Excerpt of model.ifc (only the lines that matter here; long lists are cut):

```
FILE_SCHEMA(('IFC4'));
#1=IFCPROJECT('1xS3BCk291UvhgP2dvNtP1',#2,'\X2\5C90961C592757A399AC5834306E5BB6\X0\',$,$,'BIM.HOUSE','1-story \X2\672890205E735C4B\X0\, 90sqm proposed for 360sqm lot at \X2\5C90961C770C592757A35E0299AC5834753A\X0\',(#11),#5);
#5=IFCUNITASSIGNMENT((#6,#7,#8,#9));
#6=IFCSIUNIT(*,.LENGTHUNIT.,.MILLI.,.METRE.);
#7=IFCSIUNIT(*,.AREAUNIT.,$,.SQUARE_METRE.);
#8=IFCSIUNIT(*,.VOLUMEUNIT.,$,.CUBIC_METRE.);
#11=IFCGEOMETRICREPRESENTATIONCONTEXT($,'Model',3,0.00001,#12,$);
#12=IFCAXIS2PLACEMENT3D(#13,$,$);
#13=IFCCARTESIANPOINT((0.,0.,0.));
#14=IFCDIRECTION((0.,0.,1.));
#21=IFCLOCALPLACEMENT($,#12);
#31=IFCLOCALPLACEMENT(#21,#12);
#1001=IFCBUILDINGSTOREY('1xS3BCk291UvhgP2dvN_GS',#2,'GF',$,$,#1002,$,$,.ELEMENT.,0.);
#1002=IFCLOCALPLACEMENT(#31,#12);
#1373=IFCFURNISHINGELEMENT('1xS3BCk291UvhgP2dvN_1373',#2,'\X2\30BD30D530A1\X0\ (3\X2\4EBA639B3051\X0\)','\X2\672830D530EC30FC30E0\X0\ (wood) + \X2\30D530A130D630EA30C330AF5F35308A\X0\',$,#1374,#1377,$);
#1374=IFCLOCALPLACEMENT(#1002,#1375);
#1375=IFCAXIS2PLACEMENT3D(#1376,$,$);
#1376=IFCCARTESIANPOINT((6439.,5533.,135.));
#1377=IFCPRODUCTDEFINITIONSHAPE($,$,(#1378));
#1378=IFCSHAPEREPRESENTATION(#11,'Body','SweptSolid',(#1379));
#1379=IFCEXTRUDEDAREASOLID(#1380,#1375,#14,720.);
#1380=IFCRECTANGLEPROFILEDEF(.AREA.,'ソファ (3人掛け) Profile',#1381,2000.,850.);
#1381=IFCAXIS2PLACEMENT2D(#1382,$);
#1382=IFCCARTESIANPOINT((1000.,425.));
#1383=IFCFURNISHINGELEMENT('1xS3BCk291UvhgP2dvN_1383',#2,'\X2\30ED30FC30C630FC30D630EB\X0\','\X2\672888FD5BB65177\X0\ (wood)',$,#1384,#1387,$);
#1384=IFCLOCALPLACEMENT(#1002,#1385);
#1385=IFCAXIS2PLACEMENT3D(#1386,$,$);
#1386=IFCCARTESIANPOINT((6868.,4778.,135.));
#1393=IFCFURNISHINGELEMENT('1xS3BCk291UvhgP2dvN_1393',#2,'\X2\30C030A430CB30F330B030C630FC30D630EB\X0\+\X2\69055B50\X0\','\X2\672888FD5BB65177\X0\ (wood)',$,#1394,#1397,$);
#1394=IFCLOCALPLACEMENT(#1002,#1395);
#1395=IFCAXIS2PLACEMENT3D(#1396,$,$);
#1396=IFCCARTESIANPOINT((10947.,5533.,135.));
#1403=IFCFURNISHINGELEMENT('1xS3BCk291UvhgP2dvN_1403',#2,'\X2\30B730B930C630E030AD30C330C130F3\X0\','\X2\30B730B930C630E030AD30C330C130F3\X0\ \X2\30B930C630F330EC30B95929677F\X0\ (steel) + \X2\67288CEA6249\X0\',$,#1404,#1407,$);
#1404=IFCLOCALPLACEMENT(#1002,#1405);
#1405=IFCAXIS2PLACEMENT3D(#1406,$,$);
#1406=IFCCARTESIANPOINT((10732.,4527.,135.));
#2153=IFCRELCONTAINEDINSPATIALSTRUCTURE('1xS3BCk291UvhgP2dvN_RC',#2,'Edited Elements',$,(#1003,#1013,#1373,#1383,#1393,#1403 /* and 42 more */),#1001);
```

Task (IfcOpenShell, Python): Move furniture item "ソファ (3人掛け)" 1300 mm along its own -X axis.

```python
import ifcopenshell
import ifcopenshell.api.geometry
import ifcopenshell.util.placement

model = ifcopenshell.open("model.ifc")

item = model.by_id(1373)
matrix = ifcopenshell.util.placement.get_local_placement(item.ObjectPlacement)
matrix[:3, 3] -= matrix[:3, 0] * 1300.0
ifcopenshell.api.geometry.edit_object_placement(model, product=item, matrix=matrix, is_si=False)

print(ifcopenshell.util.placement.get_local_placement(item.ObjectPlacement).round(3) + 0.0)

model.write("model_edited.ifc")
```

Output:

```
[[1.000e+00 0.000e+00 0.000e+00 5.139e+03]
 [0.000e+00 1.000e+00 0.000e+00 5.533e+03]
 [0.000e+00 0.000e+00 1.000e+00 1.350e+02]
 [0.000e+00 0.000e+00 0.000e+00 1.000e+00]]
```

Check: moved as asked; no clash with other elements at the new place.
